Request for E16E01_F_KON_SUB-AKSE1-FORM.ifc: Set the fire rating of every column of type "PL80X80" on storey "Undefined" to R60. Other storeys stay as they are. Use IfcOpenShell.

First a look at what the model holds.

```python
import ifcopenshell
import ifcopenshell.util.element

model = ifcopenshell.open("E16E01_F_KON_SUB-AKSE1-FORM.ifc")
print(model.schema)
storey = next(s for s in model.by_type("IfcBuildingStorey") if s.Name == "Undefined")
columns = [e for e in ifcopenshell.util.element.get_decomposition(storey) if e.is_a("IfcColumn")]
seen = {}
for e in columns:
    element_type = ifcopenshell.util.element.get_type(e)
    key = (element_type.Name if element_type != e and element_type else None, ifcopenshell.util.element.get_pset(e, "Pset_ColumnCommon", "FireRating"))
    seen[key] = seen.get(key, 0) + 1
for (name, value), count in sorted(seen.items(), key=str):
    print(count, "x", name, "|", value)
```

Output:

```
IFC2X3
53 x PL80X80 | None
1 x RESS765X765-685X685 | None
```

```python
import ifcopenshell
import ifcopenshell.api.pset
import ifcopenshell.util.element

model = ifcopenshell.open("E16E01_F_KON_SUB-AKSE1-FORM.ifc")

storey = next(s for s in model.by_type("IfcBuildingStorey") if s.Name == "Undefined")
columns = [e for e in ifcopenshell.util.element.get_decomposition(storey) if e.is_a("IfcColumn")]

count = 0
for e in columns:
    element_type = ifcopenshell.util.element.get_type(e)
    if element_type in (None, e) or element_type.Name != "PL80X80":
        continue
    found = ifcopenshell.util.element.get_pset(e, "Pset_ColumnCommon", should_inherit=False)
    if found:
        pset = model.by_id(found["id"])
        if len(ifcopenshell.util.element.get_elements_by_pset(pset)) > 1:
            pset = ifcopenshell.api.pset.unshare_pset(model, products=[e], pset=pset)[0]
    else:
        pset = ifcopenshell.api.pset.add_pset(model, product=e, name="Pset_ColumnCommon")
    ifcopenshell.api.pset.edit_pset(model, pset=pset, properties={"FireRating": "R60"})
    count += 1

print(count, "columns updated")

model.write("E16E01_F_KON_SUB-AKSE1-FORM-out.ifc")
```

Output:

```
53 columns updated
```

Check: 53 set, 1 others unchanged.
